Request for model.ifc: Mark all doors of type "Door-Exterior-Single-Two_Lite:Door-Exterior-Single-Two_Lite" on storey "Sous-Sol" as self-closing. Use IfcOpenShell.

First a look at what the model holds.

```python
import ifcopenshell
import ifcopenshell.util.element

model = ifcopenshell.open("model.ifc")
print(model.schema)
storey = next(s for s in model.by_type("IfcBuildingStorey") if s.Name == "Sous-Sol")
doors = [e for e in ifcopenshell.util.element.get_decomposition(storey) if e.is_a("IfcDoor")]
seen = {}
for e in doors:
    element_type = ifcopenshell.util.element.get_type(e)
    key = (element_type.Name if element_type != e and element_type else None, ifcopenshell.util.element.get_pset(e, "Pset_DoorCommon", "SelfClosing"))
    seen[key] = seen.get(key, 0) + 1
for (name, value), count in sorted(seen.items(), key=str):
    print(count, "x", name, "|", value)
```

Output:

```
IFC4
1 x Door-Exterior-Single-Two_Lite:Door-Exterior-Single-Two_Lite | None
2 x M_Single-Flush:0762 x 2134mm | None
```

```python
import ifcopenshell
import ifcopenshell.api.pset
import ifcopenshell.util.element

model = ifcopenshell.open("model.ifc")

storey = next(s for s in model.by_type("IfcBuildingStorey") if s.Name == "Sous-Sol")
doors = [e for e in ifcopenshell.util.element.get_decomposition(storey) if e.is_a("IfcDoor")]

count = 0
for e in doors:
    element_type = ifcopenshell.util.element.get_type(e)
    if element_type in (None, e) or element_type.Name != "Door-Exterior-Single-Two_Lite:Door-Exterior-Single-Two_Lite":
        continue
    # add_pset returns the element's existing set when there is one.
    pset = ifcopenshell.api.pset.add_pset(model, product=e, name="Pset_DoorCommon")
    ifcopenshell.api.pset.edit_pset(model, pset=pset, properties={"SelfClosing": True})
    count += 1

print(count, "doors updated")

model.write("model_v2.ifc")
```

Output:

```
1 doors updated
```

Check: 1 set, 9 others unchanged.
